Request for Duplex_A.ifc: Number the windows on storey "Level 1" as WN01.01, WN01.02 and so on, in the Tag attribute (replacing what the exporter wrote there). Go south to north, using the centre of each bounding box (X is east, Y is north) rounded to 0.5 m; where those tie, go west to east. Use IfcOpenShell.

First a look at what the model holds.

```python
import ifcopenshell
import ifcopenshell.util.element
import ifcopenshell.util.placement

model = ifcopenshell.open("Duplex_A.ifc")
print(model.schema)
storey = next(s for s in model.by_type("IfcBuildingStorey") if s.Name == "Level 1")
windows = [e for e in ifcopenshell.util.element.get_decomposition(storey) if e.is_a("IfcWindow")]
for e in sorted(windows, key=lambda e: e.id()):
    origin = ifcopenshell.util.placement.get_local_placement(e.ObjectPlacement)[:3, 3]
    print(e.id(), e.Tag, e.Name, origin.round(2) + 0.0, sep=" | ")
```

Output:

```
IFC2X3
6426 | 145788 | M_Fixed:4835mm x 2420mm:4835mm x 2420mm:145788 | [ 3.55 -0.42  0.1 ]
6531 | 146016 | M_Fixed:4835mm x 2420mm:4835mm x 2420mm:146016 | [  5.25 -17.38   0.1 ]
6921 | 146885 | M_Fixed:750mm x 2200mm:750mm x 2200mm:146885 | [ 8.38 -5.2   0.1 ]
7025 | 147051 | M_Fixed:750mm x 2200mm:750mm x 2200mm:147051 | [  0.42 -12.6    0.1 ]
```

```python
import ifcopenshell
import ifcopenshell.geom
import ifcopenshell.util.element
import ifcopenshell.util.shape

model = ifcopenshell.open("Duplex_A.ifc")
settings = ifcopenshell.geom.settings()
settings.set("use-world-coords", True)


def centre(element):
    shape = ifcopenshell.geom.create_shape(settings, element)
    return ifcopenshell.util.shape.get_bbox_centroid(shape.geometry)


storey = next(s for s in model.by_type("IfcBuildingStorey") if s.Name == "Level 1")
windows = [e for e in ifcopenshell.util.element.get_decomposition(storey) if e.is_a("IfcWindow")]

# Insertion points can sit at a corner or the storey origin, so sort by the geometry (in metres).
centres = {e: centre(e) for e in windows}
windows.sort(key=lambda e: (round(centres[e][1] / 0.5), centres[e][0]))

for i, e in enumerate(windows, start=1):
    number = f"WN01.{i:02d}"
    e.Tag = number
    print(e.id(), number)

model.write("Duplex_A_rev.ifc")
```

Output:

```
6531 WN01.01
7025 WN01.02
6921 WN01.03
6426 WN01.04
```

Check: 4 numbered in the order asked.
